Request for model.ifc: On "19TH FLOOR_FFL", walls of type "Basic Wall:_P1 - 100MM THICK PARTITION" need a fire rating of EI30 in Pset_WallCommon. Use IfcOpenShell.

First a look at what the model holds.

```python
import ifcopenshell
import ifcopenshell.util.element

model = ifcopenshell.open("model.ifc")
print(model.schema)
storey = next(s for s in model.by_type("IfcBuildingStorey") if s.Name == "19TH FLOOR_FFL")
walls = [e for e in ifcopenshell.util.element.get_decomposition(storey) if e.is_a("IfcWall")]
seen = {}
for e in walls:
    element_type = ifcopenshell.util.element.get_type(e)
    key = (element_type.Name if element_type != e and element_type else None, ifcopenshell.util.element.get_pset(e, "Pset_WallCommon", "FireRating"))
    seen[key] = seen.get(key, 0) + 1
for (name, value), count in sorted(seen.items(), key=str):
    print(count, "x", name, "|", value)
```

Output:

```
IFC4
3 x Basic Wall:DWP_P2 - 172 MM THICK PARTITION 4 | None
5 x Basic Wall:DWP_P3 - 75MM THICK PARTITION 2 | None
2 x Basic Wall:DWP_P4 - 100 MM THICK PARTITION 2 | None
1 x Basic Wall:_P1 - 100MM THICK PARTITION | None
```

```python
import ifcopenshell
import ifcopenshell.api.pset
import ifcopenshell.util.element

model = ifcopenshell.open("model.ifc")

storey = next(s for s in model.by_type("IfcBuildingStorey") if s.Name == "19TH FLOOR_FFL")
walls = [e for e in ifcopenshell.util.element.get_decomposition(storey) if e.is_a("IfcWall")]

count = 0
for e in walls:
    element_type = ifcopenshell.util.element.get_type(e)
    if element_type in (None, e) or element_type.Name != "Basic Wall:_P1 - 100MM THICK PARTITION":
        continue
    # add_pset returns the element's existing set when there is one.
    pset = ifcopenshell.api.pset.add_pset(model, product=e, name="Pset_WallCommon")
    ifcopenshell.api.pset.edit_pset(model, pset=pset, properties={"FireRating": "EI30"})
    count += 1

print(count, "walls updated")

model.write("model_rev.ifc")
```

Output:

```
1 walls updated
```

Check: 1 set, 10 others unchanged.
